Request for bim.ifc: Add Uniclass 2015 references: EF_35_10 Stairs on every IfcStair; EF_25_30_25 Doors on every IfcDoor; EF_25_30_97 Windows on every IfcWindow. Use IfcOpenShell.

First a look at what the model holds.

```python
import ifcopenshell

model = ifcopenshell.open("bim.ifc")
print(model.schema)
print("classifications:", [c.Name for c in model.by_type("IfcClassification")])
for ifc_class in ("IfcDoor", "IfcRoof", "IfcStair", "IfcWall", "IfcWindow"):
    print(ifc_class, len(model.by_type(ifc_class)))
```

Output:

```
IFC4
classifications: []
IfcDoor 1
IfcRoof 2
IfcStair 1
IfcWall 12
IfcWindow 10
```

```python
import ifcopenshell
import ifcopenshell.api.classification

model = ifcopenshell.open("bim.ifc")

system = ifcopenshell.api.classification.add_classification(model, classification="Uniclass 2015")

codes = {
    "IfcStair": ("EF_35_10", "Stairs"),
    "IfcDoor": ("EF_25_30_25", "Doors"),
    "IfcWindow": ("EF_25_30_97", "Windows"),
}
for ifc_class, (code, name) in codes.items():
    products = model.by_type(ifc_class)
    ifcopenshell.api.classification.add_reference(
        model, products=products, classification=system, identification=code, name=name
    )
    print(code, len(products))

model.write("bim_v2.ifc")
```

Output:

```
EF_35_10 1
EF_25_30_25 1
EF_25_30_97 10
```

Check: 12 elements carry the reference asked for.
